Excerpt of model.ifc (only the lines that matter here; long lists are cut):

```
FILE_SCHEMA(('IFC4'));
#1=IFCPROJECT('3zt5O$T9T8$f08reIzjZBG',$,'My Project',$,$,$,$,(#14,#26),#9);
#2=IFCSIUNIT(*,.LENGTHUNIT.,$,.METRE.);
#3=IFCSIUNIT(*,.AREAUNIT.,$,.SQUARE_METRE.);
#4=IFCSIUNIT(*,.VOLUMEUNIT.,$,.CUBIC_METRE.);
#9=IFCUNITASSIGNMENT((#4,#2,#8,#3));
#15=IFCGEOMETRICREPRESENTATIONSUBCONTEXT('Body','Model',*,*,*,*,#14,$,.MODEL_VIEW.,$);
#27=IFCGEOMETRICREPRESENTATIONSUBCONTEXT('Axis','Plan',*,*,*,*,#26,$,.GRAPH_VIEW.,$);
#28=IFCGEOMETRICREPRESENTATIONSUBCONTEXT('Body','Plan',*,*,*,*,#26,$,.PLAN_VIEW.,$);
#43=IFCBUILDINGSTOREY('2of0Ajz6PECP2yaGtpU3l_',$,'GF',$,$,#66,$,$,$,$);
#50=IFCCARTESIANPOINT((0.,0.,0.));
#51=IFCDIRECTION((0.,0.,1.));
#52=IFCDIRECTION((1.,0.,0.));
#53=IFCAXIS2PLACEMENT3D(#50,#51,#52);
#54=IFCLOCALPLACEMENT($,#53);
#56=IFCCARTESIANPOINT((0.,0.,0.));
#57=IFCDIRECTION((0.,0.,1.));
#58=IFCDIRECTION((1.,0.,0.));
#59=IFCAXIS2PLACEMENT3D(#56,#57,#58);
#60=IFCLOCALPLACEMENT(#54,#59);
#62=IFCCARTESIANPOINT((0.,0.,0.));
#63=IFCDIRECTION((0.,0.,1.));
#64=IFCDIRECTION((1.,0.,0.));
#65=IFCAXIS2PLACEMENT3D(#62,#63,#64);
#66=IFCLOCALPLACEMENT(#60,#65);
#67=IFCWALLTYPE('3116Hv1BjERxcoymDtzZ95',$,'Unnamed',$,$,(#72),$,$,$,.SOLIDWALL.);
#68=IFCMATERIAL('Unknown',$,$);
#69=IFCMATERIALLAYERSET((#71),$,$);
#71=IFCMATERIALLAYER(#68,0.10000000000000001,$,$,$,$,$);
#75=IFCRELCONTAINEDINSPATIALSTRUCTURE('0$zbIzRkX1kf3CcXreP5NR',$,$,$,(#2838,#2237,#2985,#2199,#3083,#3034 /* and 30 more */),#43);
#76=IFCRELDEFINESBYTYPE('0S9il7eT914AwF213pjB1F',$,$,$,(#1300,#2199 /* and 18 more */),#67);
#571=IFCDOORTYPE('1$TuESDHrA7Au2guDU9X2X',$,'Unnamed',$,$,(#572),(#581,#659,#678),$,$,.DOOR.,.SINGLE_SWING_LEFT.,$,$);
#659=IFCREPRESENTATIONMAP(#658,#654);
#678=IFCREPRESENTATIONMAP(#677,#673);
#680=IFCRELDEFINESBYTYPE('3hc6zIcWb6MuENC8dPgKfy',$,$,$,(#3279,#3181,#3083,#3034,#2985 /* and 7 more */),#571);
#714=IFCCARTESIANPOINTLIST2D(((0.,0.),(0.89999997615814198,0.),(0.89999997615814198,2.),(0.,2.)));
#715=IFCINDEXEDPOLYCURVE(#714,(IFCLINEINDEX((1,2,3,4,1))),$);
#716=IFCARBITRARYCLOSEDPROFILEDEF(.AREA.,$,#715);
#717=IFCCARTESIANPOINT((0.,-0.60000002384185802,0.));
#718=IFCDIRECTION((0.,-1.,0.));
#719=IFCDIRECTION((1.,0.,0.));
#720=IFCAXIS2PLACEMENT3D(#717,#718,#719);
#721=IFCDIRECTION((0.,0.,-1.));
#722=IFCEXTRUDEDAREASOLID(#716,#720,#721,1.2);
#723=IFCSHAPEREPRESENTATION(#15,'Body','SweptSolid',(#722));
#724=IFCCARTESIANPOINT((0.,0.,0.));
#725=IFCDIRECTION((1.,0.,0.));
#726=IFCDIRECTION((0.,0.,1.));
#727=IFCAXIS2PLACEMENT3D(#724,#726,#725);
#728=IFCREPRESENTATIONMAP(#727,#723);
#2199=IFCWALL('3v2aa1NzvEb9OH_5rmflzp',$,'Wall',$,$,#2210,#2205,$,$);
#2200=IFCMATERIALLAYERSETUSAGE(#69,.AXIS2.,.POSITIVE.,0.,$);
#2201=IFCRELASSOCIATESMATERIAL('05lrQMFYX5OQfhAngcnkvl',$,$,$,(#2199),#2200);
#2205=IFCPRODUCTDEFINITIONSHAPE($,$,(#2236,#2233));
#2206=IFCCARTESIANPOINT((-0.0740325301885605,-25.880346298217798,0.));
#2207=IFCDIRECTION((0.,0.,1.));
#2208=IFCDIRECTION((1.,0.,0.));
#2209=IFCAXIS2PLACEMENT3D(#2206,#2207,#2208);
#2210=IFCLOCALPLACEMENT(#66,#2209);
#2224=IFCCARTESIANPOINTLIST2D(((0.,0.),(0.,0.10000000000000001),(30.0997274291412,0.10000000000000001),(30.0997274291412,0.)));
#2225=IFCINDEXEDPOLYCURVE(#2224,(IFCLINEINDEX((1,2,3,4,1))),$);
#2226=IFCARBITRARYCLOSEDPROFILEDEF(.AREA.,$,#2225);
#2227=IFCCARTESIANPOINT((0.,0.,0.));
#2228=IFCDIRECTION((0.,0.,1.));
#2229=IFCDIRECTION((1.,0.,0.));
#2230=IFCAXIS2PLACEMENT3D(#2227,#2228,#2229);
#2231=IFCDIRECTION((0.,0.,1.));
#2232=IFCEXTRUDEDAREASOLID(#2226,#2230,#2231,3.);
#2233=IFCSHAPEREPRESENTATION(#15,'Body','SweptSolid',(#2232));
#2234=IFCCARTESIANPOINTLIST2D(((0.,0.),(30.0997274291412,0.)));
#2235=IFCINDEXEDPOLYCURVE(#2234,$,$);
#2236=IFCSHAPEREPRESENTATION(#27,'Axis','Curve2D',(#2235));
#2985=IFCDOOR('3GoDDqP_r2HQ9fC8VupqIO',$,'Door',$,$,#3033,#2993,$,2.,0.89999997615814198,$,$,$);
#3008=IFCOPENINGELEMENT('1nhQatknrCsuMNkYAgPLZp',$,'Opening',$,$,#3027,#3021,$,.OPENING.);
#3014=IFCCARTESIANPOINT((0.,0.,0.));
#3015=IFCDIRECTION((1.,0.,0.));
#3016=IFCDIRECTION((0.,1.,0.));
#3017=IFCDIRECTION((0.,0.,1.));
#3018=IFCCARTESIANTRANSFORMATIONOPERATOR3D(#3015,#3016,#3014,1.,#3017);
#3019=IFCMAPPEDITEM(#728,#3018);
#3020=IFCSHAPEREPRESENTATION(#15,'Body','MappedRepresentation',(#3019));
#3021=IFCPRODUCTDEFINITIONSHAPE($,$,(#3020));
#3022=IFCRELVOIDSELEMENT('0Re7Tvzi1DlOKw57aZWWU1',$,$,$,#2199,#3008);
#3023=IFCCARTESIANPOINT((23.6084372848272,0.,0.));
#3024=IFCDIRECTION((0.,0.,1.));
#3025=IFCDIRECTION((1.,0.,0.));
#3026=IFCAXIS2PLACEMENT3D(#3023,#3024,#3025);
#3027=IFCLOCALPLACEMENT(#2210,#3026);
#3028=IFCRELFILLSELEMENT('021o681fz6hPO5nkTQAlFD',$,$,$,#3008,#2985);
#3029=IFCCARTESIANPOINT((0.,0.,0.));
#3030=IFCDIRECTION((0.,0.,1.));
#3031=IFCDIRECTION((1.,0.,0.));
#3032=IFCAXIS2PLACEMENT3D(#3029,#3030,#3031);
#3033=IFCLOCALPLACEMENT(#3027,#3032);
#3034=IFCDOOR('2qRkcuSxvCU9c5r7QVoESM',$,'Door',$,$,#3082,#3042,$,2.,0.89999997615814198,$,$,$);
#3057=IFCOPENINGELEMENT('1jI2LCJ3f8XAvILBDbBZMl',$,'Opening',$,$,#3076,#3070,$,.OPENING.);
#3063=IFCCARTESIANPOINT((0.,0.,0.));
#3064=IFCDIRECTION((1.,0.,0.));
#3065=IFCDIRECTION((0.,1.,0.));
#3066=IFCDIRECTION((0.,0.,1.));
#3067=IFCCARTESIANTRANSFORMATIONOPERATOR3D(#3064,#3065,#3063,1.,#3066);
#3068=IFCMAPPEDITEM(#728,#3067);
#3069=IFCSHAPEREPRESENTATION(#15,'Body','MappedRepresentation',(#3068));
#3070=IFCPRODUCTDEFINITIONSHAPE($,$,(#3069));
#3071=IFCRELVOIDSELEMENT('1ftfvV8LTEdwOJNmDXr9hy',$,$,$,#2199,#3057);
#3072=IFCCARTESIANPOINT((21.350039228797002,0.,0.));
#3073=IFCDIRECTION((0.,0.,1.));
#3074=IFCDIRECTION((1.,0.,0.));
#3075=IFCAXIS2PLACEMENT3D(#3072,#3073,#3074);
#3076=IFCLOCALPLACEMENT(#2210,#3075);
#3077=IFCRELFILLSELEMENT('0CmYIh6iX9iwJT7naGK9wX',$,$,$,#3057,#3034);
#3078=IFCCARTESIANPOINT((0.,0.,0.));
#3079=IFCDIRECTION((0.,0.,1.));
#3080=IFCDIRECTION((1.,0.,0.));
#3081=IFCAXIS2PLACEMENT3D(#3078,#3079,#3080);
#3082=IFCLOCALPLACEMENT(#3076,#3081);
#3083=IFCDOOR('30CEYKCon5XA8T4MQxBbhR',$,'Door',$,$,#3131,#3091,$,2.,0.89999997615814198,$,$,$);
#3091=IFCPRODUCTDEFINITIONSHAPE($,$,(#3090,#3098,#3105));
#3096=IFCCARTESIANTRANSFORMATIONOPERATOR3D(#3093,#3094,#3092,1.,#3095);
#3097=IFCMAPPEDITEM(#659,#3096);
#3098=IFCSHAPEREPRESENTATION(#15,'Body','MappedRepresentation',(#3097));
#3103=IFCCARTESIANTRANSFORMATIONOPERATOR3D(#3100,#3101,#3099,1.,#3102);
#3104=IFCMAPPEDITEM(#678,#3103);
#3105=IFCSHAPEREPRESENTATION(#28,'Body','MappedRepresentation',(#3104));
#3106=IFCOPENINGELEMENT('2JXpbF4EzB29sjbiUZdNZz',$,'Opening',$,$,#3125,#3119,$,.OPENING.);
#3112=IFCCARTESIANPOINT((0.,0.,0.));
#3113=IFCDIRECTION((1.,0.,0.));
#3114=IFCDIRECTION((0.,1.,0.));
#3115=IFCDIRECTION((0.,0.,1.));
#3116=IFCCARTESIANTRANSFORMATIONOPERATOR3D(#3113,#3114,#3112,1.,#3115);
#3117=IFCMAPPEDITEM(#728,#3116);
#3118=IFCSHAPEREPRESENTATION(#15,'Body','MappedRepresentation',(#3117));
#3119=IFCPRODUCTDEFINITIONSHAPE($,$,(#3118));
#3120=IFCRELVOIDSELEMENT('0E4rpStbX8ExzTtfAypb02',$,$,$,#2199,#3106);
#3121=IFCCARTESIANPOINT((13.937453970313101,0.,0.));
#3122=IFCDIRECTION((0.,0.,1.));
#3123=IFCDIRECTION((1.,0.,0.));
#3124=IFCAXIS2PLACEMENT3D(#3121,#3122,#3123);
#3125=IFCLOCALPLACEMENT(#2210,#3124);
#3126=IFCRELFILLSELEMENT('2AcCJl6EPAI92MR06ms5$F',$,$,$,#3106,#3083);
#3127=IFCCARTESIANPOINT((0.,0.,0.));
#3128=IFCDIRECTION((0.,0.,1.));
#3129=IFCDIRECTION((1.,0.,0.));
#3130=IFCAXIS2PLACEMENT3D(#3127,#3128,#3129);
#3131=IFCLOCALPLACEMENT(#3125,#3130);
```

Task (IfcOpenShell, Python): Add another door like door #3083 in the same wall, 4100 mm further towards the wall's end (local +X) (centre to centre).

```python
import ifcopenshell
import ifcopenshell.api.feature
import ifcopenshell.api.geometry
import ifcopenshell.api.root
import ifcopenshell.geom
import ifcopenshell.util.element
import ifcopenshell.util.placement
import ifcopenshell.util.shape
import ifcopenshell.util.unit

model = ifcopenshell.open("model.ifc")
unit_scale = ifcopenshell.util.unit.calculate_unit_scale(model)
settings = ifcopenshell.geom.settings()


def volume(element):
    """Net volume in cubic metres, openings subtracted."""
    shape = ifcopenshell.geom.create_shape(settings, element)
    return ifcopenshell.util.shape.get_volume(shape.geometry)


door = model.by_guid("30CEYKCon5XA8T4MQxBbhR")
opening = door.FillsVoids[0].RelatingOpeningElement
wall = opening.VoidsElements[0].RelatingBuildingElement
before = volume(wall)
shift = ifcopenshell.util.placement.get_local_placement(wall.ObjectPlacement)[:3, 0] * 4.1 / unit_scale

# copy_class copies the void relationship, type, container and properties, but no geometry.
new_opening = ifcopenshell.api.root.copy_class(model, product=opening)
new_opening.Representation = ifcopenshell.util.element.copy_deep(
    model, opening.Representation, exclude=["IfcGeometricRepresentationContext", "IfcRepresentationMap"]
)
new_door = ifcopenshell.api.root.copy_class(model, product=door)
new_door.Representation = ifcopenshell.util.element.copy_deep(
    model, door.Representation, exclude=["IfcGeometricRepresentationContext", "IfcRepresentationMap"]
)
ifcopenshell.api.feature.add_filling(model, opening=new_opening, element=new_door)

for old, new in ((opening, new_opening), (door, new_door)):
    matrix = ifcopenshell.util.placement.get_local_placement(old.ObjectPlacement)
    matrix[:3, 3] += shift
    ifcopenshell.api.geometry.edit_object_placement(model, product=new, matrix=matrix, is_si=False)

after = volume(wall)

print(f"wall volume {before:.3f} -> {after:.3f} m3")

model.write("model_updated.ifc")
```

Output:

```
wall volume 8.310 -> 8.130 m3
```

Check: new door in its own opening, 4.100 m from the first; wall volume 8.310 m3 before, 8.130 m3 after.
